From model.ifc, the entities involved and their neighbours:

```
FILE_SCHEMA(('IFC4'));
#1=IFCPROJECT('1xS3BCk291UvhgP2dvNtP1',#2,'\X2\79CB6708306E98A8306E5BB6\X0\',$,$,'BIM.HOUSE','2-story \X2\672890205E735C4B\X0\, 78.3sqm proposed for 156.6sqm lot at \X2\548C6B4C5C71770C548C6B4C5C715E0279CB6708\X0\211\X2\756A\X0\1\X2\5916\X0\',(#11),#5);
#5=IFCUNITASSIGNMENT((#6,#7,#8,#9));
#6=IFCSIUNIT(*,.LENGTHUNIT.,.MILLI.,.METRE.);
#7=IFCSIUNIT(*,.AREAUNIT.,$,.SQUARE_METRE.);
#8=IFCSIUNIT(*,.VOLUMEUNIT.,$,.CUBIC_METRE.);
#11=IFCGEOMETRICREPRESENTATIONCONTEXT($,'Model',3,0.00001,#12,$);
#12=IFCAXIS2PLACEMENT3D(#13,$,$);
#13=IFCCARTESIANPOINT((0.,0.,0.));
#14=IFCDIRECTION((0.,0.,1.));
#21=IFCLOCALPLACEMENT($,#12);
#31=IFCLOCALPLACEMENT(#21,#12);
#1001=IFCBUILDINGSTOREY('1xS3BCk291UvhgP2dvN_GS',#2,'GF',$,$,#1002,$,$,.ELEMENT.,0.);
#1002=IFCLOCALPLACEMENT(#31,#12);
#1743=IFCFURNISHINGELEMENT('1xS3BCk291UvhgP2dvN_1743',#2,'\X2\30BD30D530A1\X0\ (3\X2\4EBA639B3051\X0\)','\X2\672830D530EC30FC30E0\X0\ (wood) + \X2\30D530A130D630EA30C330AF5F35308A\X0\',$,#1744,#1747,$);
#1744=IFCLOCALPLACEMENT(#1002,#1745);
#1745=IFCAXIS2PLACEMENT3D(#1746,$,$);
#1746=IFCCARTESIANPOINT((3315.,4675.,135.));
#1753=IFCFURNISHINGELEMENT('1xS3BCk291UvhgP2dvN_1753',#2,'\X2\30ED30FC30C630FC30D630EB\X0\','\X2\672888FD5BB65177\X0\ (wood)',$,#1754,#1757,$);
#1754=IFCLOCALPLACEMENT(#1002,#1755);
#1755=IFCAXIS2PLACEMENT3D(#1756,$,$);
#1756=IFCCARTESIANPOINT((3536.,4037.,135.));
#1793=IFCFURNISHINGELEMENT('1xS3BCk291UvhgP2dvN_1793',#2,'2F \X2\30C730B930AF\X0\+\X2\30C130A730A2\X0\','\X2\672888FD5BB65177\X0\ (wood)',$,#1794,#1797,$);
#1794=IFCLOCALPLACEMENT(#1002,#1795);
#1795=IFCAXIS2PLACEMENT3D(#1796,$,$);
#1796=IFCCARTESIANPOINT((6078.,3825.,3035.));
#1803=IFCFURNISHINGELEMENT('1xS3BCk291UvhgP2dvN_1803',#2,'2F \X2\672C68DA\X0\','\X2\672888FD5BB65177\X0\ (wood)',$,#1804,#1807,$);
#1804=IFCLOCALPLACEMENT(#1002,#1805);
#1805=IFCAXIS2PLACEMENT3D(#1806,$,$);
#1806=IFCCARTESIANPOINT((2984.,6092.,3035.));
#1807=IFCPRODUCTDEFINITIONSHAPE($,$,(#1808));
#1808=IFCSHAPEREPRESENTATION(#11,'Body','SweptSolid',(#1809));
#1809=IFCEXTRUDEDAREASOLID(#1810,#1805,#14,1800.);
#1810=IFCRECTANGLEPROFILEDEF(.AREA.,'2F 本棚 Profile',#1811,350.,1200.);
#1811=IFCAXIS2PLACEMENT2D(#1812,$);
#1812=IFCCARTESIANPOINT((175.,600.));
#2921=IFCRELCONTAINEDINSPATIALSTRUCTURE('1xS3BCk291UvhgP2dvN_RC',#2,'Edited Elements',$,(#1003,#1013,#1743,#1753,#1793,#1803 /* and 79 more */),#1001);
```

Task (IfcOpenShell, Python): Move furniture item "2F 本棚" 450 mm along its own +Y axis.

```python
import ifcopenshell
import ifcopenshell.api.geometry
import ifcopenshell.util.placement

model = ifcopenshell.open("model.ifc")

item = model.by_guid("1xS3BCk291UvhgP2dvN_1803")
matrix = ifcopenshell.util.placement.get_local_placement(item.ObjectPlacement)
matrix[:3, 3] += matrix[:3, 1] * 450.0
ifcopenshell.api.geometry.edit_object_placement(model, product=item, matrix=matrix, is_si=False)

print(ifcopenshell.util.placement.get_local_placement(item.ObjectPlacement).round(3) + 0.0)

model.write("model_edited.ifc")
```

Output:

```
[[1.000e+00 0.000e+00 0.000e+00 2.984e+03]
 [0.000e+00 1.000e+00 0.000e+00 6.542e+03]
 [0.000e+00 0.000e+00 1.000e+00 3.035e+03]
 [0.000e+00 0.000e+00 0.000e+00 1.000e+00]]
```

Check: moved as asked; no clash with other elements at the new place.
